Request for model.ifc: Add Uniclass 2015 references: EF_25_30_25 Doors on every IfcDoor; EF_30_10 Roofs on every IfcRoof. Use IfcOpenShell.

First a look at what the model holds.

```python
import ifcopenshell

model = ifcopenshell.open("model.ifc")
print(model.schema)
print("classifications:", [c.Name for c in model.by_type("IfcClassification")])
for ifc_class in ("IfcDoor", "IfcRoof", "IfcStair", "IfcWall", "IfcWindow"):
    print(ifc_class, len(model.by_type(ifc_class)))
```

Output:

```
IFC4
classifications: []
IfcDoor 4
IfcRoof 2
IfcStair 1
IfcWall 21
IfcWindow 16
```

```python
import ifcopenshell
import ifcopenshell.api.classification

model = ifcopenshell.open("model.ifc")

system = ifcopenshell.api.classification.add_classification(model, classification="Uniclass 2015")

codes = {
    "IfcDoor": ("EF_25_30_25", "Doors"),
    "IfcRoof": ("EF_30_10", "Roofs"),
}
for ifc_class, (code, name) in codes.items():
    products = model.by_type(ifc_class)
    ifcopenshell.api.classification.add_reference(
        model, products=products, classification=system, identification=code, name=name
    )
    print(code, len(products))

model.write("model_rev.ifc")
```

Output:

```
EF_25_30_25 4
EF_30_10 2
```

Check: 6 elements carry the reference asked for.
